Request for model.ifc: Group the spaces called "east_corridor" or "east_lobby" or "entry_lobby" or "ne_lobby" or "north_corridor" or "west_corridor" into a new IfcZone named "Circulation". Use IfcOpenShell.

First a look at what the model holds.

```python
import ifcopenshell

model = ifcopenshell.open("model.ifc")
print(model.schema)
seen = {}
for space in model.by_type("IfcSpace"):
    seen[space.Name] = seen.get(space.Name, 0) + 1
for name, count in sorted(seen.items(), key=str):
    print(count, "x", name)
print("zones:", [z.Name for z in model.by_type("IfcZone")][:20])
```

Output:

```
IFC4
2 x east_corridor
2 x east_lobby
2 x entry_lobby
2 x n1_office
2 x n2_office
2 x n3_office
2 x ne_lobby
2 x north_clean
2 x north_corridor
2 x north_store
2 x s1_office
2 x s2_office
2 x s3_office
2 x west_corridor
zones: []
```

```python
import ifcopenshell
import ifcopenshell.api.group
import ifcopenshell.api.root

model = ifcopenshell.open("model.ifc")

names = {"east_corridor", "east_lobby", "entry_lobby", "ne_lobby", "north_corridor", "west_corridor"}
spaces = [s for s in model.by_type("IfcSpace") if s.Name in names]

zone = ifcopenshell.api.root.create_entity(model, ifc_class="IfcZone", name="Circulation")
ifcopenshell.api.group.assign_group(model, products=spaces, group=zone)
print(len(spaces), "spaces in", zone.Name)

model.write("model_rev.ifc")
```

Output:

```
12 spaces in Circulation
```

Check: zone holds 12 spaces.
